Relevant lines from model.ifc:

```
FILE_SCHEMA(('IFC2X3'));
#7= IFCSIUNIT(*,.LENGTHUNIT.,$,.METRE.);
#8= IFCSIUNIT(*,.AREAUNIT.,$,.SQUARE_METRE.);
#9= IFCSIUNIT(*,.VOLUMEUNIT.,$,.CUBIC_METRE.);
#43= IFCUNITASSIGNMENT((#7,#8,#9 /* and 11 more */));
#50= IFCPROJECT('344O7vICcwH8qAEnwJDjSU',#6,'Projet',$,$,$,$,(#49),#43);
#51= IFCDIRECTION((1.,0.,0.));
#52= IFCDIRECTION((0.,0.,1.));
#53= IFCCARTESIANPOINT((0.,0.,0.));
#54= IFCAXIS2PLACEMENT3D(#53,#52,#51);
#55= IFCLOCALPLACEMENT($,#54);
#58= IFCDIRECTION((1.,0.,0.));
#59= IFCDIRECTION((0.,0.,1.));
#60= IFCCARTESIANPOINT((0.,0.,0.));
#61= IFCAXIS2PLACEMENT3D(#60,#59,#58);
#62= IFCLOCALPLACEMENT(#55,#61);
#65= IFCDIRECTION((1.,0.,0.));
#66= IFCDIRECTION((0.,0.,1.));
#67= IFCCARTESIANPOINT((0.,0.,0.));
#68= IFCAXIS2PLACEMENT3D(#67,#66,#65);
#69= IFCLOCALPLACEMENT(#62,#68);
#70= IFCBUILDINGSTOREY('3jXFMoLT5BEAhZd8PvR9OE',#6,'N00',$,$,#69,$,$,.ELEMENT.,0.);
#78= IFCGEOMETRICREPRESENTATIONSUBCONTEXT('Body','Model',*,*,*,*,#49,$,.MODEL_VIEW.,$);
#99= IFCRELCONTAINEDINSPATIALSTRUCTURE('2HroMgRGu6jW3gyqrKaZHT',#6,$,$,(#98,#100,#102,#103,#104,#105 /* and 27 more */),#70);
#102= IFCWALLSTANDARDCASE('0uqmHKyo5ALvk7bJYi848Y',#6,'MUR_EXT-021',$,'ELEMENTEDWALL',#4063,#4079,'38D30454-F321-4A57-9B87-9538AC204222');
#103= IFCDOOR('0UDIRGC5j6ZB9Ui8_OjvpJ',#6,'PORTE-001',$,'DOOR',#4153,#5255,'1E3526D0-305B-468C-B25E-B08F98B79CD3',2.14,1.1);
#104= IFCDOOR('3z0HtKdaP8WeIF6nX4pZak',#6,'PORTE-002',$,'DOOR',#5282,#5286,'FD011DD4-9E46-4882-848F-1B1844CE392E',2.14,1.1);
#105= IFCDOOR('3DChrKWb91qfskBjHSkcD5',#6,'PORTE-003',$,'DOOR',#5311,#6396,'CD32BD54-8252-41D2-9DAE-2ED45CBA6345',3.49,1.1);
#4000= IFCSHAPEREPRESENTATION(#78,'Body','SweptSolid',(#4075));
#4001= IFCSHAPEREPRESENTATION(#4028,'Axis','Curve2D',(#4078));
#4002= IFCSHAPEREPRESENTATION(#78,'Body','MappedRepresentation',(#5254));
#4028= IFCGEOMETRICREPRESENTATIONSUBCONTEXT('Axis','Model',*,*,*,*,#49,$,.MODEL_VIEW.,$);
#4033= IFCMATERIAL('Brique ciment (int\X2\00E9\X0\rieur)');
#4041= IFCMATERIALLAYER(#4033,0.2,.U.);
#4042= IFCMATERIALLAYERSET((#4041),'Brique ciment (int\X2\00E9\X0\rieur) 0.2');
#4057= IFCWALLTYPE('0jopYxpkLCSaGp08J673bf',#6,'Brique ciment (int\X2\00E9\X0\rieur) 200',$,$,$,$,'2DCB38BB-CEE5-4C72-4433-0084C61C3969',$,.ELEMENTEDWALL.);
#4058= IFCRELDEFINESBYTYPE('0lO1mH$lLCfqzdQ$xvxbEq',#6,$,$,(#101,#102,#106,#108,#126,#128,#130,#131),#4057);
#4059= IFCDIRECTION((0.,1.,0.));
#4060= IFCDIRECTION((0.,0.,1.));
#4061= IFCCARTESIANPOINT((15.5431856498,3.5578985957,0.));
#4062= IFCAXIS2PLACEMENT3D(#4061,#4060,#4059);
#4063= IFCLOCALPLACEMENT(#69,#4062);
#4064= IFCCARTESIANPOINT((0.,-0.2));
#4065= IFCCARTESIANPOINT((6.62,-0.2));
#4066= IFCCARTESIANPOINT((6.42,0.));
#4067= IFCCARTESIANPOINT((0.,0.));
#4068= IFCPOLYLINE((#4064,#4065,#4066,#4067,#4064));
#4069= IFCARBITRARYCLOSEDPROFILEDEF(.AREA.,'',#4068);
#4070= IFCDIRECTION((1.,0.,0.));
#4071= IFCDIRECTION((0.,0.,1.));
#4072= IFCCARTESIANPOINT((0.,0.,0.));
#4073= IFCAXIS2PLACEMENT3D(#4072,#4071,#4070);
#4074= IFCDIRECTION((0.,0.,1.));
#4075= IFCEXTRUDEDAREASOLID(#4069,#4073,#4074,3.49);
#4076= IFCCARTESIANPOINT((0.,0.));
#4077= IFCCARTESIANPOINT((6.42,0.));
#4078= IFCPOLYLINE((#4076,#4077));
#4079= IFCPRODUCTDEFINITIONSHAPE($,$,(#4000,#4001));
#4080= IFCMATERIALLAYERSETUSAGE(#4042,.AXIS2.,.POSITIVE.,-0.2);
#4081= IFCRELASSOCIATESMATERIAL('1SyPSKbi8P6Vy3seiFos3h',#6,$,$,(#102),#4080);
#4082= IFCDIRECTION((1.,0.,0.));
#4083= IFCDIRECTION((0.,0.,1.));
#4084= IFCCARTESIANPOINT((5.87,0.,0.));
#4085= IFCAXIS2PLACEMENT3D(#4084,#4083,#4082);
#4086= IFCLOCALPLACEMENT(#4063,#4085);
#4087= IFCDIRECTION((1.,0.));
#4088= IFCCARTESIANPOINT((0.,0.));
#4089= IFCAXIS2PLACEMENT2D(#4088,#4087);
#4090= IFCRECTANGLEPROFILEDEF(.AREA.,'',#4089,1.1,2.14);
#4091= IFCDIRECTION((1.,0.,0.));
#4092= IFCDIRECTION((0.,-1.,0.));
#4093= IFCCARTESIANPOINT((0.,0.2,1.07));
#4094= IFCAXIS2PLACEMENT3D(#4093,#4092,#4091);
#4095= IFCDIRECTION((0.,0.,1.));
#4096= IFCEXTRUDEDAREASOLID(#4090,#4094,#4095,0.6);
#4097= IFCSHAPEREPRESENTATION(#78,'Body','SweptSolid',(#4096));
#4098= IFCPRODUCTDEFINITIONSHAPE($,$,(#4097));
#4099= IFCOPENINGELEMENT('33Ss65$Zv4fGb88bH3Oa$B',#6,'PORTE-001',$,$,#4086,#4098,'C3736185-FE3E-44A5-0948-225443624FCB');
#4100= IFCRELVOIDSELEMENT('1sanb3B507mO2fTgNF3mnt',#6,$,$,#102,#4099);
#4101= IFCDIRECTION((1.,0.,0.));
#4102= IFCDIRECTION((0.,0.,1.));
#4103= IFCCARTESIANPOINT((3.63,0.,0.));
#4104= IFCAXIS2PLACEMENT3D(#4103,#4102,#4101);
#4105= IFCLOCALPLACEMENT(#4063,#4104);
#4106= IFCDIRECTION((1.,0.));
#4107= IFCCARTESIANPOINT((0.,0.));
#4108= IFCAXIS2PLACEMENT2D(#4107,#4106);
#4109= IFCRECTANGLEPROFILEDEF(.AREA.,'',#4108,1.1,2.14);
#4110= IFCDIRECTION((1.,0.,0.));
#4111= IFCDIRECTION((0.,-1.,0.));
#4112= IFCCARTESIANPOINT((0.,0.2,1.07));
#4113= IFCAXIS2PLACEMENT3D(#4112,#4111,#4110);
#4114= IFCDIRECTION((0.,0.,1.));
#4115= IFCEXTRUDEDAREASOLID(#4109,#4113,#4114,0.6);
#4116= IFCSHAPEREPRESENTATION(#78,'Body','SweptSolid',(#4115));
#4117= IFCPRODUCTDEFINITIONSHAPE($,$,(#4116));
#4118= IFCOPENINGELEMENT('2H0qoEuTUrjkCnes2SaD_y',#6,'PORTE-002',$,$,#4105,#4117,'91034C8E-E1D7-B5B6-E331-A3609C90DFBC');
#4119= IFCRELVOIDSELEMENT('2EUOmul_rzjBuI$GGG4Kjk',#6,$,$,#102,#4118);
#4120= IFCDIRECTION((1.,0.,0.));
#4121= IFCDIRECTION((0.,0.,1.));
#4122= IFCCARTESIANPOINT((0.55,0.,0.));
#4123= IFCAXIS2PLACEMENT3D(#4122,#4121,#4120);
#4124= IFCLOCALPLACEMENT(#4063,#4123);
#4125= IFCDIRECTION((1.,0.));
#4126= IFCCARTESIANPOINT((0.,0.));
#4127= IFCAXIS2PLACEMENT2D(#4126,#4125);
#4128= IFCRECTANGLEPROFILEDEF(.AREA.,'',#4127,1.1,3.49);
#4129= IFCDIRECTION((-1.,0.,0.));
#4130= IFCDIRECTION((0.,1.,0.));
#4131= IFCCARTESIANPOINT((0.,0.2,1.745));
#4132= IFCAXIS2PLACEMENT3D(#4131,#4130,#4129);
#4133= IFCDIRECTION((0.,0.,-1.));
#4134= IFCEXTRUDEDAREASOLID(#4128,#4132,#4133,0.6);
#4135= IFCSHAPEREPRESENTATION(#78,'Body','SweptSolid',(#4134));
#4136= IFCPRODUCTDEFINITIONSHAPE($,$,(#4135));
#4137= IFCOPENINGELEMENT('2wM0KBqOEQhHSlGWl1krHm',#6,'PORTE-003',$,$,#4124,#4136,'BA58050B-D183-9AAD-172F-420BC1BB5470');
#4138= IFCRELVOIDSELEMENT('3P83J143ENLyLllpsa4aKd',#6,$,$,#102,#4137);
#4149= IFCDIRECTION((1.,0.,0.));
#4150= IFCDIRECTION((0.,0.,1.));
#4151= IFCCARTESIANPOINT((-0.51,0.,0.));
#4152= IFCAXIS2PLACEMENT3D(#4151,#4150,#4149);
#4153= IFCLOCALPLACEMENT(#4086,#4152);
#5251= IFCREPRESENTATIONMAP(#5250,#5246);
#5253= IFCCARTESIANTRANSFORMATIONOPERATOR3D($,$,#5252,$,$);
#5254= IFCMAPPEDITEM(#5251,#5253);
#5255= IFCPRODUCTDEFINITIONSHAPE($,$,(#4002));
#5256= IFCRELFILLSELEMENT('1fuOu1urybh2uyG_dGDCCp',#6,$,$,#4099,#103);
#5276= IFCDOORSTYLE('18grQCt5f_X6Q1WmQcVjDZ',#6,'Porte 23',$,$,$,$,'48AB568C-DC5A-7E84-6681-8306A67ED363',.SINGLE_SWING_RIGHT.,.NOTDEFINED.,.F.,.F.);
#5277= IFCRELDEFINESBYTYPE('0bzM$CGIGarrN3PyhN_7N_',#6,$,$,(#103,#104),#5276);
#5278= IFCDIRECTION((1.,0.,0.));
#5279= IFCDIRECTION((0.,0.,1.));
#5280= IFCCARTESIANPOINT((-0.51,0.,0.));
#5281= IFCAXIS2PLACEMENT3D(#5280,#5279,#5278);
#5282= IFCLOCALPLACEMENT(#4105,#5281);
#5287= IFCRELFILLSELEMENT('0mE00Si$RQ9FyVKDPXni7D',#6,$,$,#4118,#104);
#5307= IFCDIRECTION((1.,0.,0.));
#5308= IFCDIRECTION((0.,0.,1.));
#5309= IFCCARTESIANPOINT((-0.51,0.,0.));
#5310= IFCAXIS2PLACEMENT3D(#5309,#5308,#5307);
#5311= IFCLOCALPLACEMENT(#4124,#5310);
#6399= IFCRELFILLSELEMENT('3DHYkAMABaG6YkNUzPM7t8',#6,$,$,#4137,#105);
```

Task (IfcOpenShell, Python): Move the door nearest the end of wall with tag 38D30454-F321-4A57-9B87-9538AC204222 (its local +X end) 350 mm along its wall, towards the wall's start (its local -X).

```python
import ifcopenshell
import ifcopenshell.api.geometry
import ifcopenshell.util.placement
import ifcopenshell.util.unit

model = ifcopenshell.open("model.ifc")
unit_scale = ifcopenshell.util.unit.calculate_unit_scale(model)

door = model.by_guid("0UDIRGC5j6ZB9Ui8_OjvpJ")
opening = door.FillsVoids[0].RelatingOpeningElement
wall = opening.VoidsElements[0].RelatingBuildingElement

wall_matrix = ifcopenshell.util.placement.get_local_placement(wall.ObjectPlacement)
shift = wall_matrix[:3, 0] * -0.35 / unit_scale
before = ifcopenshell.util.placement.get_local_placement(door.ObjectPlacement)[:3, 3].copy()

# The door is placed relative to its opening, so it follows when the opening moves.
matrix = ifcopenshell.util.placement.get_local_placement(opening.ObjectPlacement)
matrix[:3, 3] += shift
ifcopenshell.api.geometry.edit_object_placement(
    model, product=opening, matrix=matrix, is_si=False, should_transform_children=True
)

after = ifcopenshell.util.placement.get_local_placement(door.ObjectPlacement)[:3, 3]
print("door moved by", (after - before).round(3) + 0.0)

model.write("model-out.ifc")
```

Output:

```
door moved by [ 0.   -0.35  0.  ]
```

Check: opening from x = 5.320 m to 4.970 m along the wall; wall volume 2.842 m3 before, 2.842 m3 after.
